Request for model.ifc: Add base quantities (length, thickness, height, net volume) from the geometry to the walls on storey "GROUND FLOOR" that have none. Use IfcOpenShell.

First a look at what the model holds.

```python
import ifcopenshell
import ifcopenshell.util.element
import ifcopenshell.util.unit

model = ifcopenshell.open("model.ifc")
print(model.schema)
for unit_type in ("LENGTHUNIT", "AREAUNIT", "VOLUMEUNIT"):
    print(unit_type, ifcopenshell.util.unit.calculate_unit_scale(model, unit_type))
storey = next(s for s in model.by_type("IfcBuildingStorey") if s.Name == "GROUND FLOOR")
walls = [e for e in ifcopenshell.util.element.get_decomposition(storey) if e.is_a("IfcWall")]
for e in sorted(walls, key=lambda e: e.id()):
    print(e.id(), e.is_a(), e.Name, list(ifcopenshell.util.element.get_psets(e, qtos_only=True)), sep=" | ")
```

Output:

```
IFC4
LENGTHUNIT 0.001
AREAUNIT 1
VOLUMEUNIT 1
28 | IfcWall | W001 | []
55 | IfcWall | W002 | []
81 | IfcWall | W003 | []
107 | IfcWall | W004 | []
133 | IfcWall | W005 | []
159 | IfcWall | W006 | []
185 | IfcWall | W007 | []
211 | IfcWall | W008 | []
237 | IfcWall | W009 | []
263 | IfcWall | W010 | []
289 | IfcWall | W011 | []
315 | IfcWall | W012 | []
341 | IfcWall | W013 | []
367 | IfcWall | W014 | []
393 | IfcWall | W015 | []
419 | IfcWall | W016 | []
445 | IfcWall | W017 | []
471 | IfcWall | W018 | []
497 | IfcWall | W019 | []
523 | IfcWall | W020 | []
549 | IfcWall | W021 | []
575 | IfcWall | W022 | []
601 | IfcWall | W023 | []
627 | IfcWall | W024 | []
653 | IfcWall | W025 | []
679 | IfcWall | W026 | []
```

```python
import ifcopenshell
import ifcopenshell.api.pset
import ifcopenshell.geom
import ifcopenshell.util.element
import ifcopenshell.util.shape
import ifcopenshell.util.unit

model = ifcopenshell.open("model.ifc")
unit_scale = ifcopenshell.util.unit.calculate_unit_scale(model)
volume_scale = ifcopenshell.util.unit.calculate_unit_scale(model, "VOLUMEUNIT")
settings = ifcopenshell.geom.settings()

storey = next(s for s in model.by_type("IfcBuildingStorey") if s.Name == "GROUND FLOOR")
walls = [e for e in ifcopenshell.util.element.get_decomposition(storey) if e.is_a("IfcWall")]

for e in sorted(walls, key=lambda e: e.id()):
    if ifcopenshell.util.element.get_psets(e, qtos_only=True, should_inherit=False):
        continue
    # Geometry comes back in metres, in the element's own axes.
    shape = ifcopenshell.geom.create_shape(settings, e)
    values = {
        "Length": ifcopenshell.util.shape.get_x(shape.geometry) / unit_scale,
        "Width": ifcopenshell.util.shape.get_y(shape.geometry) / unit_scale,
        "Height": ifcopenshell.util.shape.get_z(shape.geometry) / unit_scale,
        "NetVolume": ifcopenshell.util.shape.get_volume(shape.geometry) / volume_scale,
    }
    qto = ifcopenshell.api.pset.add_qto(model, product=e, name="Qto_WallBaseQuantities")
    ifcopenshell.api.pset.edit_qto(model, qto=qto, properties=values)
    print(e.id(), {k: round(v, 3) for k, v in values.items()})

model.write("model_updated.ifc")
```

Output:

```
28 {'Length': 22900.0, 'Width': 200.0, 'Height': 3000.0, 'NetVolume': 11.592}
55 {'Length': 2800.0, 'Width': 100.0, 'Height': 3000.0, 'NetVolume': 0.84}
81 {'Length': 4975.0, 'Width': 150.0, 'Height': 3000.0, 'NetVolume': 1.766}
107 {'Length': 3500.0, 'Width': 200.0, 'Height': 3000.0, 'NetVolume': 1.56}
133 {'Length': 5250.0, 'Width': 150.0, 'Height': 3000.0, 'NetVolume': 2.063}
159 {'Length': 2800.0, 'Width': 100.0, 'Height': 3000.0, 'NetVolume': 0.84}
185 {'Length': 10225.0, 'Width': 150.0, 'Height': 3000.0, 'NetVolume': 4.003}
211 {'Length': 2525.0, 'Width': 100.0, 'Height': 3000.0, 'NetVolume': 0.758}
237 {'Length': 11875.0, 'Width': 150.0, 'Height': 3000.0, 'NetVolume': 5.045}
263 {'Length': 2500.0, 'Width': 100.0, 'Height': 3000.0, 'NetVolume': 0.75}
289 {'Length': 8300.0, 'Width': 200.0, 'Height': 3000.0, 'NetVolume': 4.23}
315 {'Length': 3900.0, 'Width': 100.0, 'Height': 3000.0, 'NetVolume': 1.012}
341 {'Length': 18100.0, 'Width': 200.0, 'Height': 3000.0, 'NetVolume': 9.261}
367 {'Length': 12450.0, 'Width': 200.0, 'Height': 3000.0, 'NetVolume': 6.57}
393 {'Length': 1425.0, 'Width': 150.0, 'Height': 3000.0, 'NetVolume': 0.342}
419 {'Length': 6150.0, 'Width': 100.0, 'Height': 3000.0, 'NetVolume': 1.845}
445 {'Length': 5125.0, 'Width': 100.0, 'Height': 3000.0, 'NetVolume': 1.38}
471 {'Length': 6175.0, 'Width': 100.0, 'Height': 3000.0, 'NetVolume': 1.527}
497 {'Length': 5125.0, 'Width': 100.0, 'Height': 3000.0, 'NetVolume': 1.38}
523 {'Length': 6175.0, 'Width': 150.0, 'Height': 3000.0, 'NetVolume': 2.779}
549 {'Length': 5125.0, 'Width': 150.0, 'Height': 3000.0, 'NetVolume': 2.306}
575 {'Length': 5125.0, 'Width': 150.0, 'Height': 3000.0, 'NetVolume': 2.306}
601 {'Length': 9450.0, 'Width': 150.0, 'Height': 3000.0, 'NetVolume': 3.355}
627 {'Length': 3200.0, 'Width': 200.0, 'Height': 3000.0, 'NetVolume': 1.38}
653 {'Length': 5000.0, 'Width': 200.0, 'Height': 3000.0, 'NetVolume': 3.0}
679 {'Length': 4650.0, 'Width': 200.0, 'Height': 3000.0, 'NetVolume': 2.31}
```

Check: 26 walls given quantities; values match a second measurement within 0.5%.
